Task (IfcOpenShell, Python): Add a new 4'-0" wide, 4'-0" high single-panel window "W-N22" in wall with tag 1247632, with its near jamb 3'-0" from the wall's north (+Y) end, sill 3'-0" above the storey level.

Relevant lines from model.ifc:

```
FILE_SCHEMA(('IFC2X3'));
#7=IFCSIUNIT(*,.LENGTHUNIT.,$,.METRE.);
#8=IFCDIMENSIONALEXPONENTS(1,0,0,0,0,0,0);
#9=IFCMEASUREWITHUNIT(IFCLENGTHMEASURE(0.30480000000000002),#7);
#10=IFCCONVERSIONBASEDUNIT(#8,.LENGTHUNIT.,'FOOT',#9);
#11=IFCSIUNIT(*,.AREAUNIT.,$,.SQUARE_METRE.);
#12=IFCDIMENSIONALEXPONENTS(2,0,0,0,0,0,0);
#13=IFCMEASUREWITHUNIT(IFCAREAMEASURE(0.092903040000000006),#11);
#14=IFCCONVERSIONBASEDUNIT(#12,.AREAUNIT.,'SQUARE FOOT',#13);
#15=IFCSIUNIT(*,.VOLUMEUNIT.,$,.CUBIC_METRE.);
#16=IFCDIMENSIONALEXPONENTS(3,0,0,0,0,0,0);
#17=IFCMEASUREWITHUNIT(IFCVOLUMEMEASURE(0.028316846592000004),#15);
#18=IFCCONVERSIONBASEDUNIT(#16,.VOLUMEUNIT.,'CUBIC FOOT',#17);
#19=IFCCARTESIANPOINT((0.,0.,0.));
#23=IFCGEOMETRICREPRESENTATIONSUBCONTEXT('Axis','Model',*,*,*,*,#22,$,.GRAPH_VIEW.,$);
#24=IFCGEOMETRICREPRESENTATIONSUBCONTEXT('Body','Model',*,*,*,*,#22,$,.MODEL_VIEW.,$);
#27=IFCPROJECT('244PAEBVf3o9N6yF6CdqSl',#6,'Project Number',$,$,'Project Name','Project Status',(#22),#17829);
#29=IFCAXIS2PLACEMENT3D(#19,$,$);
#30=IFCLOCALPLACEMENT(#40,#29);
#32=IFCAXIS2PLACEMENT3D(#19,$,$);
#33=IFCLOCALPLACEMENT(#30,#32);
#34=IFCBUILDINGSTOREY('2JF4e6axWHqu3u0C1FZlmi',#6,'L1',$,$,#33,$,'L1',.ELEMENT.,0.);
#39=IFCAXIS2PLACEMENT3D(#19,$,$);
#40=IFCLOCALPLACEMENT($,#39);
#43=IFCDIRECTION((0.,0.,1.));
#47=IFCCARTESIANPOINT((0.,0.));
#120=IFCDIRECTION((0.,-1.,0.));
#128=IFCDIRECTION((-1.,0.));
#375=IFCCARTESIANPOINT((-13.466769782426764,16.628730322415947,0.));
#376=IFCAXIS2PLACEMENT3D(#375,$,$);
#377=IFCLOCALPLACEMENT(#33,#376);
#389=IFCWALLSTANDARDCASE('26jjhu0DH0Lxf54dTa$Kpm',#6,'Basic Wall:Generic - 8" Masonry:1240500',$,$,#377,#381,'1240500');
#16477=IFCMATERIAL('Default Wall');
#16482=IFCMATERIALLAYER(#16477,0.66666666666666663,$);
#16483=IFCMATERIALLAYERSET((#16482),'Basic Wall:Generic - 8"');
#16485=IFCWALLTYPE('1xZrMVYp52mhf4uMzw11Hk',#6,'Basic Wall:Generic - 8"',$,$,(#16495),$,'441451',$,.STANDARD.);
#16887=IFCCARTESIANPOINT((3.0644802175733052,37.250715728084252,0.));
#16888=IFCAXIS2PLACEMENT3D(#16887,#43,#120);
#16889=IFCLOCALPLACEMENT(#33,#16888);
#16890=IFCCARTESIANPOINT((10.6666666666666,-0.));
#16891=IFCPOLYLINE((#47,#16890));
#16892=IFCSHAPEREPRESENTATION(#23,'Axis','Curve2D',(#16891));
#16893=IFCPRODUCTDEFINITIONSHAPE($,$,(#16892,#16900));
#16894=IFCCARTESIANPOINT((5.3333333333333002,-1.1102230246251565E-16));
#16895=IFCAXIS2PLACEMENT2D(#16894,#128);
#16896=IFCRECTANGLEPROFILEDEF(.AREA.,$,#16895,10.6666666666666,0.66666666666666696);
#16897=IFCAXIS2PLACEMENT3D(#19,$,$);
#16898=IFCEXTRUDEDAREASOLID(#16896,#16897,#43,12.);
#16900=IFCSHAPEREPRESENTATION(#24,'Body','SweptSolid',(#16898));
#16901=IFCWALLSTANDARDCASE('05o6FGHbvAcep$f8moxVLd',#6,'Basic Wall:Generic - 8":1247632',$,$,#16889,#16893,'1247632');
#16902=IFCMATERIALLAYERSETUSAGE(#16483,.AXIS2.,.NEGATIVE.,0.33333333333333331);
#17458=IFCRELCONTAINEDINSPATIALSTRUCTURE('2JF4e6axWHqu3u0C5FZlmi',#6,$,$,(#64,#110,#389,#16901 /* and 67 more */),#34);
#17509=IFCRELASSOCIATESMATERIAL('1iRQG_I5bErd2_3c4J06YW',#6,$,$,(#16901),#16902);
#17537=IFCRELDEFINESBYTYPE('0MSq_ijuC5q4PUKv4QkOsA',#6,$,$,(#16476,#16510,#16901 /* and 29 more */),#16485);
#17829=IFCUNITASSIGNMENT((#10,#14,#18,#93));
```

```python
import numpy as np
import ifcopenshell
import ifcopenshell.api.feature
import ifcopenshell.api.geometry
import ifcopenshell.api.root
import ifcopenshell.api.spatial
import ifcopenshell.api.type
import ifcopenshell.geom
import ifcopenshell.util.element
import ifcopenshell.util.placement
import ifcopenshell.util.representation
import ifcopenshell.util.shape
import ifcopenshell.util.unit

model = ifcopenshell.open("model.ifc")
unit_scale = ifcopenshell.util.unit.calculate_unit_scale(model)
settings = ifcopenshell.geom.settings()


def volume(element):
    """Net volume in cubic metres, openings subtracted."""
    shape = ifcopenshell.geom.create_shape(settings, element)
    return ifcopenshell.util.shape.get_volume(shape.geometry)


wall = model.by_guid("05o6FGHbvAcep$f8moxVLd")
storey = ifcopenshell.util.element.get_container(wall, ifc_class="IfcBuildingStorey")
context = ifcopenshell.util.representation.get_context(model, "Model", "Body", "MODEL_VIEW")
before = volume(wall)

width, height, from_end, sill = 1.2192, 1.2192, 0.9144, 0.9144  # metres

# The wall runs along its own X axis, and the end named is its -X end.
wall_shape = ifcopenshell.geom.create_shape(settings, wall)
x, y, z = ifcopenshell.util.shape.get_vertices(wall_shape.geometry).T
start = x.min() + from_end
face, thickness = float(y.min()), float(y.max() - y.min())
wall_matrix = ifcopenshell.util.placement.get_local_placement(wall.ObjectPlacement)
level = ifcopenshell.util.placement.get_local_placement(storey.ObjectPlacement)[2, 3]


def in_wall(x, y):
    """Placement at x, y metres in the wall's axes, at sill height."""
    matrix = wall_matrix.copy()
    matrix[:, 3] = wall_matrix @ np.array([x / unit_scale, y / unit_scale, 0.0, 1.0])
    matrix[2, 3] = level + sill / unit_scale
    return matrix


# Opening: a box that overshoots both wall faces by 50 mm.
opening = ifcopenshell.api.root.create_entity(model, ifc_class="IfcOpeningElement")
box = ifcopenshell.api.geometry.add_wall_representation(
    model, context=context, length=width, height=height, thickness=thickness + 0.1
)
ifcopenshell.api.geometry.assign_representation(model, product=opening, representation=box)
ifcopenshell.api.geometry.edit_object_placement(model, product=opening, matrix=in_wall(start, face - 0.05), is_si=False)
ifcopenshell.api.feature.add_feature(model, feature=opening, element=wall)

window = ifcopenshell.api.root.create_entity(model, ifc_class="IfcWindow", name="W-N22")
window.OverallWidth, window.OverallHeight = width / unit_scale, height / unit_scale
body = ifcopenshell.api.geometry.add_window_representation(
    model,
    context=context,
    overall_width=window.OverallWidth,
    overall_height=window.OverallHeight,
    partition_type="SINGLE_PANEL",
)
ifcopenshell.api.geometry.assign_representation(model, product=window, representation=body)
ifcopenshell.api.spatial.assign_container(model, products=[window], relating_structure=storey)
fills = ifcopenshell.api.feature.add_filling(model, opening=opening, element=window)
fills.OwnerHistory = window.OwnerHistory  # required in IFC2X3

# IFC2X3 keeps the operation on the window style.
style = ifcopenshell.api.root.create_entity(model, ifc_class="IfcWindowStyle", name="W-N22")
style.OperationType, style.ConstructionType = "SINGLE_PANEL", "NOTDEFINED"
style.ParameterTakesPrecedence = style.Sizeable = False
ifcopenshell.api.type.assign_type(model, related_objects=[window], relating_type=style)

# Centre the window in the wall's thickness.
ifcopenshell.api.geometry.edit_object_placement(model, product=window, matrix=in_wall(start, face), is_si=False)
window_shape = ifcopenshell.geom.create_shape(settings, window)
depth = ifcopenshell.util.shape.get_vertices(window_shape.geometry)[:, 1]
offset = face + thickness / 2 - (depth.min() + depth.max()) / 2
ifcopenshell.api.geometry.edit_object_placement(model, product=window, matrix=in_wall(start, offset), is_si=False)

after = volume(wall)

print(f"wall volume {before:.3f} -> {after:.3f} m3")

model.write("model_rev.ifc")
```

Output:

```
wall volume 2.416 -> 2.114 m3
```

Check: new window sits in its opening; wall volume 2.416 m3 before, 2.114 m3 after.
